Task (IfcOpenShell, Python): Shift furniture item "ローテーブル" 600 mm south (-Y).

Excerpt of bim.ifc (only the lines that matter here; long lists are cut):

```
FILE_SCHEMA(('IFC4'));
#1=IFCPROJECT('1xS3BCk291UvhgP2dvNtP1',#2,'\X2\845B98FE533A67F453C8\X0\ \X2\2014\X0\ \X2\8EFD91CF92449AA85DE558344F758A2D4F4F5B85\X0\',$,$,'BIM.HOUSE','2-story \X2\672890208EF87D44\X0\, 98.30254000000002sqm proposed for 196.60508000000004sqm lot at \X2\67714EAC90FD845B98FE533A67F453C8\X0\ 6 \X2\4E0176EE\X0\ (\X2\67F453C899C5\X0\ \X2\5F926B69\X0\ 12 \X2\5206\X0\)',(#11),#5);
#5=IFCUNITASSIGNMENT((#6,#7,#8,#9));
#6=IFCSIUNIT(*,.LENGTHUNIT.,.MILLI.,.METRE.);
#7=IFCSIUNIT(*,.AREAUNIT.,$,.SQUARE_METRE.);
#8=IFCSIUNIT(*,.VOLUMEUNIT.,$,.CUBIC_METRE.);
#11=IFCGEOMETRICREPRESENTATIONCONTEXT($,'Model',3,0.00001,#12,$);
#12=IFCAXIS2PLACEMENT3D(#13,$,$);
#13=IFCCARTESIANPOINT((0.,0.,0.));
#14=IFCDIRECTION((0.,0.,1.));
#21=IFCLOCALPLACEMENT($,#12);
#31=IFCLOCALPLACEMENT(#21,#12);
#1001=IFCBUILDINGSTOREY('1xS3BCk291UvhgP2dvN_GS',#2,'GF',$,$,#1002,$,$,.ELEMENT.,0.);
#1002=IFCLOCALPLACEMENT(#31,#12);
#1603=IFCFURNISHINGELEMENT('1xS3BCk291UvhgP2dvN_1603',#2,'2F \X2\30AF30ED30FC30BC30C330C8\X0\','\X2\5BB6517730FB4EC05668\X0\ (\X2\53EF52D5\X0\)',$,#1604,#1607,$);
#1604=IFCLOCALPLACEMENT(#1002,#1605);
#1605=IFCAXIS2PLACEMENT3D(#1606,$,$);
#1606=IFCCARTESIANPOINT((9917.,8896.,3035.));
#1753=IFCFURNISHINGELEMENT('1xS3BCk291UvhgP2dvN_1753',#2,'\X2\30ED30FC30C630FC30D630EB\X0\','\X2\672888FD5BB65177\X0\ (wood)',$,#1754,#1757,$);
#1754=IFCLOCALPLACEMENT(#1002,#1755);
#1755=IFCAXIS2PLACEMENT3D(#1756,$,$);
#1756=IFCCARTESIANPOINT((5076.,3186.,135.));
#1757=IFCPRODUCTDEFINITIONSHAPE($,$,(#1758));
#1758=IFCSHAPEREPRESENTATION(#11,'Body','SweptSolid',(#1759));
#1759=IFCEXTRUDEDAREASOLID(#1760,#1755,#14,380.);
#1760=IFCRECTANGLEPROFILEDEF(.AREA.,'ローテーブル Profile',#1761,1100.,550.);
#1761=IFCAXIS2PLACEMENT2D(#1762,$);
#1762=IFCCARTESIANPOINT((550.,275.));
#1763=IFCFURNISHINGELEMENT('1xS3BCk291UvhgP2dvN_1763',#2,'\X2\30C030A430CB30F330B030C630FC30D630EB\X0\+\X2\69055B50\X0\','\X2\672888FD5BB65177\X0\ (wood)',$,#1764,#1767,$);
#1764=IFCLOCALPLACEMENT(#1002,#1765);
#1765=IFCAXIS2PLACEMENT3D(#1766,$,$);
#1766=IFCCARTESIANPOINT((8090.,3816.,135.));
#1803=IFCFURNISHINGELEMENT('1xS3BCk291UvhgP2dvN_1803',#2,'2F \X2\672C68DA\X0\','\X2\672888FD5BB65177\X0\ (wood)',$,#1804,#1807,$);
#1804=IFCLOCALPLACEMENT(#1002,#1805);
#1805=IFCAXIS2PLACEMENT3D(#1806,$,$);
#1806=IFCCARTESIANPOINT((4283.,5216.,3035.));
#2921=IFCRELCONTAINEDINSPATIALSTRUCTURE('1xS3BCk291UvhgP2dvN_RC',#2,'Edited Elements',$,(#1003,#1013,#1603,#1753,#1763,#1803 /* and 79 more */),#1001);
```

```python
import ifcopenshell
import ifcopenshell.api.geometry
import ifcopenshell.util.placement
import ifcopenshell.util.unit

model = ifcopenshell.open("bim.ifc")
unit_scale = ifcopenshell.util.unit.calculate_unit_scale(model)

item = model.by_guid("1xS3BCk291UvhgP2dvN_1753")
matrix = ifcopenshell.util.placement.get_local_placement(item.ObjectPlacement)
matrix[1, 3] -= 0.6 / unit_scale
ifcopenshell.api.geometry.edit_object_placement(model, product=item, matrix=matrix, is_si=False)

print(ifcopenshell.util.placement.get_local_placement(item.ObjectPlacement).round(3) + 0.0)

model.write("bim-out.ifc")
```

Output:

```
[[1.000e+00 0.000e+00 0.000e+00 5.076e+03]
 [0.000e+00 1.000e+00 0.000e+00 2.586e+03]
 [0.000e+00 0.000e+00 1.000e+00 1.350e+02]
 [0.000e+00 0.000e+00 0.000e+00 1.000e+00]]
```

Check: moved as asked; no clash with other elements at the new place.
